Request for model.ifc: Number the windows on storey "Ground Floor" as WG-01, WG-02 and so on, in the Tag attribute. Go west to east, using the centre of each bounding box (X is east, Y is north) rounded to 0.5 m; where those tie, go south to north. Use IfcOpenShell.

First a look at what the model holds.

```python
import ifcopenshell
import ifcopenshell.util.element
import ifcopenshell.util.placement

model = ifcopenshell.open("model.ifc")
print(model.schema)
storey = next(s for s in model.by_type("IfcBuildingStorey") if s.Name == "Ground Floor")
windows = [e for e in ifcopenshell.util.element.get_decomposition(storey) if e.is_a("IfcWindow")]
for e in sorted(windows, key=lambda e: e.id()):
    origin = ifcopenshell.util.placement.get_local_placement(e.ObjectPlacement)[:3, 3]
    print(e.id(), e.Tag, e.Name, origin.round(2) + 0.0, sep=" | ")
```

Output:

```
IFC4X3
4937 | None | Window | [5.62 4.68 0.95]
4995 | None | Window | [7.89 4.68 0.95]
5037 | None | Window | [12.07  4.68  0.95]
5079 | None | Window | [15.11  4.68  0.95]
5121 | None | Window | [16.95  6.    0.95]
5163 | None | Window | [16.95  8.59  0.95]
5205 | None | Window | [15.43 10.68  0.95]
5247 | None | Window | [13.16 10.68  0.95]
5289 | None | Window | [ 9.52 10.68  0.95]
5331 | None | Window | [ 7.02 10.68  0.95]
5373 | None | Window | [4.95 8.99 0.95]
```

```python
import ifcopenshell
import ifcopenshell.geom
import ifcopenshell.util.element
import ifcopenshell.util.shape

model = ifcopenshell.open("model.ifc")
settings = ifcopenshell.geom.settings()
settings.set("use-world-coords", True)


def centre(element):
    shape = ifcopenshell.geom.create_shape(settings, element)
    return ifcopenshell.util.shape.get_bbox_centroid(shape.geometry)


storey = next(s for s in model.by_type("IfcBuildingStorey") if s.Name == "Ground Floor")
windows = [e for e in ifcopenshell.util.element.get_decomposition(storey) if e.is_a("IfcWindow")]

# Insertion points can sit at a corner or the storey origin, so sort by the geometry (in metres).
centres = {e: centre(e) for e in windows}
windows.sort(key=lambda e: (round(centres[e][0] / 0.5), centres[e][1]))

for i, e in enumerate(windows, start=1):
    number = f"WG-{i:02d}"
    e.Tag = number
    print(e.id(), number)

model.write("model_updated.ifc")
```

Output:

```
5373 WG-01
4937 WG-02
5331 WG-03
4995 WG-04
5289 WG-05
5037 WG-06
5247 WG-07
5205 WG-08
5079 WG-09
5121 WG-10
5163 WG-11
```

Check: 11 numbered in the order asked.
